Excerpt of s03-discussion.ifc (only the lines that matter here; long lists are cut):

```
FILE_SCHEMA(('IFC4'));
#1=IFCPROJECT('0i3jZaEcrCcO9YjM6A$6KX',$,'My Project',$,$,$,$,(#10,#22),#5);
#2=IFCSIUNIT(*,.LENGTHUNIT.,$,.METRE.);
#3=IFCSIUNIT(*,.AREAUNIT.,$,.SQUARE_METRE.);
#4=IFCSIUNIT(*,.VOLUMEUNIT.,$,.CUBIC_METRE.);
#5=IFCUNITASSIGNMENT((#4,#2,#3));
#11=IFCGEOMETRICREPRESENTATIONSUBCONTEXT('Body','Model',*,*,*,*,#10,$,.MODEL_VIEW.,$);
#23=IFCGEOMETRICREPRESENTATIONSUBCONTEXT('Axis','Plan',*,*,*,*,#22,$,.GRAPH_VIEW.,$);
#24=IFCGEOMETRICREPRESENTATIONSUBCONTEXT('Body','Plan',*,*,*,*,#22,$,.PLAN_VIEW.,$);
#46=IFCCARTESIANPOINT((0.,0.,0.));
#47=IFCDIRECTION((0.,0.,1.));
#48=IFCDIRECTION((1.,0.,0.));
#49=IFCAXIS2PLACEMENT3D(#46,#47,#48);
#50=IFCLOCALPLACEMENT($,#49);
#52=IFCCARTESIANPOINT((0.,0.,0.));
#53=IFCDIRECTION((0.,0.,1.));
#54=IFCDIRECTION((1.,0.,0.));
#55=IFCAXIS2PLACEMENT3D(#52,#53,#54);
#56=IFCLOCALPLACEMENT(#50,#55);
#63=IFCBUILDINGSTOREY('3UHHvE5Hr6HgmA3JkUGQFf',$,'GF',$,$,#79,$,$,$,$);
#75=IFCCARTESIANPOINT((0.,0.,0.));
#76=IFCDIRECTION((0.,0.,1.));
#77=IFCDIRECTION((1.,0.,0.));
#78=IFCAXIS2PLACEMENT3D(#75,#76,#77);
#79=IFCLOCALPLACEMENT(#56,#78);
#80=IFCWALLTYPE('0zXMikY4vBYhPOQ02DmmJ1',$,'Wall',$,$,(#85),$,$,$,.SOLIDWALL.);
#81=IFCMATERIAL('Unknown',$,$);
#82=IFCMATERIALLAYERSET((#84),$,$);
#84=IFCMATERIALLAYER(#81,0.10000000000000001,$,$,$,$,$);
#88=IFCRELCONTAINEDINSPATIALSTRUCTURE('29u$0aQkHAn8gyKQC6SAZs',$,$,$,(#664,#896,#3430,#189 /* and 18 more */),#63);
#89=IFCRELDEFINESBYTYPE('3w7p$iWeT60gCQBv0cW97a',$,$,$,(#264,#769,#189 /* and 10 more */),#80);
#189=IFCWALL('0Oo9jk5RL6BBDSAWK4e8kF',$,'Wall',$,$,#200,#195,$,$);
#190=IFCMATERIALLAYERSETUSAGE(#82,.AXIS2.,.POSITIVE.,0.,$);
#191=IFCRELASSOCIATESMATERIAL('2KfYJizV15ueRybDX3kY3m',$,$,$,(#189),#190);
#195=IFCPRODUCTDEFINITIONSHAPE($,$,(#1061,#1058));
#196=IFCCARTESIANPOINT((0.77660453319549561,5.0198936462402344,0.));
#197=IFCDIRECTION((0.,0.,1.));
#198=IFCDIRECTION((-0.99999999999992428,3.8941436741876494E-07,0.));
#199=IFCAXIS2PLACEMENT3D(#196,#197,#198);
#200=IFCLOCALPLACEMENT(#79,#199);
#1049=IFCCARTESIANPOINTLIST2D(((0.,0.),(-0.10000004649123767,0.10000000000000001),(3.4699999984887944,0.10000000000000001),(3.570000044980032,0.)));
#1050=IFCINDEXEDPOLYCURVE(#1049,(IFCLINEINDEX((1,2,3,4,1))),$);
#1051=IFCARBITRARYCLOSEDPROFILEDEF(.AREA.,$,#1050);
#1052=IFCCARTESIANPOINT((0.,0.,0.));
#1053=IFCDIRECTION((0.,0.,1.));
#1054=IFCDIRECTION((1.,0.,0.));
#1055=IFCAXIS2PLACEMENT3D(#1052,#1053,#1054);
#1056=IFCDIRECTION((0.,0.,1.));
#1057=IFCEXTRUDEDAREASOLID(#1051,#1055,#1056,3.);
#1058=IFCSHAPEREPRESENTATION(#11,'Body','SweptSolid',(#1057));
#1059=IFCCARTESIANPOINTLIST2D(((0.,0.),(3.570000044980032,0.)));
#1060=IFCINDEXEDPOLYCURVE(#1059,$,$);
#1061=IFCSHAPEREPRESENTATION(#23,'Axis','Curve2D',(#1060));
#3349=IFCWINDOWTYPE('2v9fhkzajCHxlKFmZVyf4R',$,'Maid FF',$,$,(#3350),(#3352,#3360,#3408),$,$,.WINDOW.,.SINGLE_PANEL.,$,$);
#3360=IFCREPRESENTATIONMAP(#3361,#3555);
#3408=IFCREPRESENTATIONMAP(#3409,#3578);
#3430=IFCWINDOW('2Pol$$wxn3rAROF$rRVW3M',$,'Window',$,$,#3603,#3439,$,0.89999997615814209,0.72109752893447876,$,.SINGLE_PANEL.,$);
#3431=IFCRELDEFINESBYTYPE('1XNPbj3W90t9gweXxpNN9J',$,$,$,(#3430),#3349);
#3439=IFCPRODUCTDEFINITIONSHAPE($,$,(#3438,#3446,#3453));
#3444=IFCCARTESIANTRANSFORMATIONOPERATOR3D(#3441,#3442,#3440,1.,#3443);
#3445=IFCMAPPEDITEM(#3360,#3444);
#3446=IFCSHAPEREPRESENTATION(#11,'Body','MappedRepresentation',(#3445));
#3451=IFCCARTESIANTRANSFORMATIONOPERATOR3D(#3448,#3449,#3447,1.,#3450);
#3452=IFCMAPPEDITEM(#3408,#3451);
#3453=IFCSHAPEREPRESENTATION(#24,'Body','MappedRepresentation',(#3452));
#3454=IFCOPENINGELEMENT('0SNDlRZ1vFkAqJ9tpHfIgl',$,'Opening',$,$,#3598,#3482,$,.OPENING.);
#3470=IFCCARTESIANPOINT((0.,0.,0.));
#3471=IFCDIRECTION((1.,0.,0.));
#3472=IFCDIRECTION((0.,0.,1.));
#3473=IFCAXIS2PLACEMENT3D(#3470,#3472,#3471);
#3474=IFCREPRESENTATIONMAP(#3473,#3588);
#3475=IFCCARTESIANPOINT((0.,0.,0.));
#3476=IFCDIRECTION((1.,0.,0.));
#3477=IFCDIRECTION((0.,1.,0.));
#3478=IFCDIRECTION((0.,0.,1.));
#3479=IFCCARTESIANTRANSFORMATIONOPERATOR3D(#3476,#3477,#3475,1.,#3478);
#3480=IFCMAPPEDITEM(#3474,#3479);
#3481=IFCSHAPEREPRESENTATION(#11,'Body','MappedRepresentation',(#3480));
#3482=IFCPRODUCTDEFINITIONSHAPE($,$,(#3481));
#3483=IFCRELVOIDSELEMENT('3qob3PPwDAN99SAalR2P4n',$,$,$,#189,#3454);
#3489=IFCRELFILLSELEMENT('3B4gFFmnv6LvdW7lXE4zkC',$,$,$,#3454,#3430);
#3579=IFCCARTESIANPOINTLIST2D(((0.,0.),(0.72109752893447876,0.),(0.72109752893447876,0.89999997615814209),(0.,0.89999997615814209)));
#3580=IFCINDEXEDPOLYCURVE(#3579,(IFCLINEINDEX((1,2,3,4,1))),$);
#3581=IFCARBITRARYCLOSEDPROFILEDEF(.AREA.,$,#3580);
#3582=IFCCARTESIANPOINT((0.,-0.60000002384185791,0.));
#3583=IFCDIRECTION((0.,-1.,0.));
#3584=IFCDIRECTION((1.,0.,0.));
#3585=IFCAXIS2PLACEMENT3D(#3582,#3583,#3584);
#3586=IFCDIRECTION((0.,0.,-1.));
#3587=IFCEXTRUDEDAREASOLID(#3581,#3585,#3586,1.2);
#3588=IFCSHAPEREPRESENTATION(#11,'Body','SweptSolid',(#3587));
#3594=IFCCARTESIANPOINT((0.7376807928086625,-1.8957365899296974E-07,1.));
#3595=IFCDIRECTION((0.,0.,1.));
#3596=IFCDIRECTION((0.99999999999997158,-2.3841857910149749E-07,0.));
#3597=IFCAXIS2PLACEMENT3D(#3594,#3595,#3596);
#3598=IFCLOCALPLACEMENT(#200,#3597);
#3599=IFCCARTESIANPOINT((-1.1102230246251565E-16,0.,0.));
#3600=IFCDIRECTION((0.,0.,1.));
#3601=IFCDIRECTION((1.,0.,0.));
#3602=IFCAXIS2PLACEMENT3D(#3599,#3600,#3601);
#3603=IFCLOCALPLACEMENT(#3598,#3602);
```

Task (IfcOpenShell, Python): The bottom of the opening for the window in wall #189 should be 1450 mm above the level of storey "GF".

```python
import numpy as np
import ifcopenshell
import ifcopenshell.api.geometry
import ifcopenshell.geom
import ifcopenshell.util.element
import ifcopenshell.util.placement
import ifcopenshell.util.shape
import ifcopenshell.util.unit

model = ifcopenshell.open("s03-discussion.ifc")
unit_scale = ifcopenshell.util.unit.calculate_unit_scale(model)

window = model.by_id(3430)
opening = window.FillsVoids[0].RelatingOpeningElement
storey = ifcopenshell.util.element.get_container(window, ifc_class="IfcBuildingStorey")
level = ifcopenshell.util.placement.get_local_placement(storey.ObjectPlacement)[2, 3]

# The opening's origin need not be at the sill, so measure its lowest point.
shape = ifcopenshell.geom.create_shape(ifcopenshell.geom.settings(), opening)
bottom = ifcopenshell.util.shape.get_shape_bottom_elevation(shape, shape.geometry) / unit_scale
dz = level + 1.45 - bottom

shift = np.array([0.0, 0.0, dz])
# The window is placed relative to its opening, so it follows when the opening moves.
matrix = ifcopenshell.util.placement.get_local_placement(opening.ObjectPlacement)
matrix[:3, 3] += shift
ifcopenshell.api.geometry.edit_object_placement(
    model, product=opening, matrix=matrix, is_si=False, should_transform_children=True
)

print(f"moved by {dz * unit_scale:+.3f} m")

model.write("s03-discussion_rev.ifc")
```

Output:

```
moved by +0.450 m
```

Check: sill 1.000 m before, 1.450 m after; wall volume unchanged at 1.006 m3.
